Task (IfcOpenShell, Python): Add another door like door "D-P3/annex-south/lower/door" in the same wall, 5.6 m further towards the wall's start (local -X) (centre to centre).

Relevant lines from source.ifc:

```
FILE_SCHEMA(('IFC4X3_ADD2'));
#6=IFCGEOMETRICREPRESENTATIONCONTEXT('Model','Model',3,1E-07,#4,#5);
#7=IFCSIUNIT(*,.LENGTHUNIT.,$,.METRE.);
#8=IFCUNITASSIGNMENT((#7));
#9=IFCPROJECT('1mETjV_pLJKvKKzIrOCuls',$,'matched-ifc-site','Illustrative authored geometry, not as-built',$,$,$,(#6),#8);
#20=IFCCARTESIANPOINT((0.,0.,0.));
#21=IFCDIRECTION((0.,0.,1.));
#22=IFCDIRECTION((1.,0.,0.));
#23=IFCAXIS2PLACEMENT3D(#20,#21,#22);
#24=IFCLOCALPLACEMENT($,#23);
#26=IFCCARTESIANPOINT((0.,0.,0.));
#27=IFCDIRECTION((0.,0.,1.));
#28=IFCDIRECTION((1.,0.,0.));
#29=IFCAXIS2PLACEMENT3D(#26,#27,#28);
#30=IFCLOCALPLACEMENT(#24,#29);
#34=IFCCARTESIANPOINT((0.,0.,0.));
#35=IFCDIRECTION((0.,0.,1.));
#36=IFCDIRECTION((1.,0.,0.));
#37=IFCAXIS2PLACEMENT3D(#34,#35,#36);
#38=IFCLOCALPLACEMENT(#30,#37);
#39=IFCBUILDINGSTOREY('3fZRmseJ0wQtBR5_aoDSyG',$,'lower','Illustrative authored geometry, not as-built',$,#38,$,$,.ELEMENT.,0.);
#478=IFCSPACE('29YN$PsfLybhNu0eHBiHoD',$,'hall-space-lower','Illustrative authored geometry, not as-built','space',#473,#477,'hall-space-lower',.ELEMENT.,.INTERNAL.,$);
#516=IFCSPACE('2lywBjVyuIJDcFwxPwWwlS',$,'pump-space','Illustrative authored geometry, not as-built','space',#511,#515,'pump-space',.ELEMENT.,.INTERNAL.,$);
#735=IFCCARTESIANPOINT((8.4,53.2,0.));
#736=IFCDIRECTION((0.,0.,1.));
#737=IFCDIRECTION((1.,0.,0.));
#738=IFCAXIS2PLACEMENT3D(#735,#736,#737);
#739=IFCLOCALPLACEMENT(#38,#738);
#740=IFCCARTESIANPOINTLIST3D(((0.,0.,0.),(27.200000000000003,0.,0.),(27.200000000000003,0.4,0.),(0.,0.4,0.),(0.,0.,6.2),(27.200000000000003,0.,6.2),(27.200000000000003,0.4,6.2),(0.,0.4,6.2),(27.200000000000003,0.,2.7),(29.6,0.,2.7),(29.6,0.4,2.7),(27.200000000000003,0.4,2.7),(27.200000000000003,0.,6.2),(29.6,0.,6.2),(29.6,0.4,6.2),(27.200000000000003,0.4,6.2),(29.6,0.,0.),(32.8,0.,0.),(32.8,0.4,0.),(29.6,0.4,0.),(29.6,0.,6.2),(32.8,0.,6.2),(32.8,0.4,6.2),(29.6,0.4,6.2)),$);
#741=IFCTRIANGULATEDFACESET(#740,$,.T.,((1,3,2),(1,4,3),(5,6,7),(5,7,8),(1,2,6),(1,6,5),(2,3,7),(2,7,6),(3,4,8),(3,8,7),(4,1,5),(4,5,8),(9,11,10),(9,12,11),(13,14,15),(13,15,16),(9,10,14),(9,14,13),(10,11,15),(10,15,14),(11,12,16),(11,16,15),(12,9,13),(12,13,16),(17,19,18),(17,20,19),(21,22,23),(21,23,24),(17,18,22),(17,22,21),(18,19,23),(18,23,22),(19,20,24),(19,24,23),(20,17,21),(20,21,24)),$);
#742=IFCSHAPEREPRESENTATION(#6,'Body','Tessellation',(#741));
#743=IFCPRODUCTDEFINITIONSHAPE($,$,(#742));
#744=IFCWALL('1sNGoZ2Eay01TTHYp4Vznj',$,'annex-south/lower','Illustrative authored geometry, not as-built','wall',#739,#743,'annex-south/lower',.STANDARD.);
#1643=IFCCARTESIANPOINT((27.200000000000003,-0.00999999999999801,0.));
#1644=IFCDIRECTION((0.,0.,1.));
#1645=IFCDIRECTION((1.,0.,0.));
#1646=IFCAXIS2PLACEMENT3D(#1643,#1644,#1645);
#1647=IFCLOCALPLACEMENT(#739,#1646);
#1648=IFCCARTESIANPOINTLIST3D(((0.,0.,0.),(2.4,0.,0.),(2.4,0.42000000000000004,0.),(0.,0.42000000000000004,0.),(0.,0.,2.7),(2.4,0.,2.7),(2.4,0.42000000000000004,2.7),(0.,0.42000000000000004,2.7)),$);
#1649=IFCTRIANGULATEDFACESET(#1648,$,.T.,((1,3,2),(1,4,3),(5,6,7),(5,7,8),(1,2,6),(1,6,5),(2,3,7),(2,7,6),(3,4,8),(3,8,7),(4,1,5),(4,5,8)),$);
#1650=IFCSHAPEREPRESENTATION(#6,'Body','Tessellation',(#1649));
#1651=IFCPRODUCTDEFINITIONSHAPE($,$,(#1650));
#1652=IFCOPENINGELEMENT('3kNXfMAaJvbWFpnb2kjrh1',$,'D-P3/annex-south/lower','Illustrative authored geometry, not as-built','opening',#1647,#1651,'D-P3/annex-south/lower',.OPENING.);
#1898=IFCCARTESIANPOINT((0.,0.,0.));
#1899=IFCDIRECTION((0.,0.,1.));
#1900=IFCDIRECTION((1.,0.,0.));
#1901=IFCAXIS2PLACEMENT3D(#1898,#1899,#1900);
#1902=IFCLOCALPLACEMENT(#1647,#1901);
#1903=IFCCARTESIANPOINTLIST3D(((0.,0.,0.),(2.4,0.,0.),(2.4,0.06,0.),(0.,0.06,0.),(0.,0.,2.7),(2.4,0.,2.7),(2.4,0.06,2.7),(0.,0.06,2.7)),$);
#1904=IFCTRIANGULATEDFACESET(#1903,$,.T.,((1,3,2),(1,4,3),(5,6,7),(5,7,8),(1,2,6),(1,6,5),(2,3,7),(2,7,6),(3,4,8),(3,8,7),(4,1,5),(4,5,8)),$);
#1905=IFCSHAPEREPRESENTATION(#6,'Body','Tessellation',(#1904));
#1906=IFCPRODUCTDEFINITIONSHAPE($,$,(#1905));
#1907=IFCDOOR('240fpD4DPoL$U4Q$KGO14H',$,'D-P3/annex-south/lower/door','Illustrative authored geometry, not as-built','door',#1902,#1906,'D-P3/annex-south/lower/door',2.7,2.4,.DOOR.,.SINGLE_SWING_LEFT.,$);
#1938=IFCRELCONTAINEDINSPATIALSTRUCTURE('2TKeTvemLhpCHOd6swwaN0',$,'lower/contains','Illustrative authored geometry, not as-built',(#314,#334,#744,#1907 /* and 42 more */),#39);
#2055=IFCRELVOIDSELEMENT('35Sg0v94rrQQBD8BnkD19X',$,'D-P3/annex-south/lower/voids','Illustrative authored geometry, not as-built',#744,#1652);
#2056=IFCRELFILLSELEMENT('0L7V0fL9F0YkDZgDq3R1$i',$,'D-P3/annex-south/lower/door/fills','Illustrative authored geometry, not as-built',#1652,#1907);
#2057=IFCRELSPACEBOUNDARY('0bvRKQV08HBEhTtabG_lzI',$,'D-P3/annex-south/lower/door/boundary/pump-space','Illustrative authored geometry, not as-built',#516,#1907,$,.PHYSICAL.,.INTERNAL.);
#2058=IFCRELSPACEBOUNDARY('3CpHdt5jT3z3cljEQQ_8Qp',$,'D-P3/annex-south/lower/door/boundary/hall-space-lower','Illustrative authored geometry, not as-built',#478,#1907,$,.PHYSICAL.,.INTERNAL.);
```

```python
import ifcopenshell
import ifcopenshell.api.feature
import ifcopenshell.api.geometry
import ifcopenshell.api.root
import ifcopenshell.geom
import ifcopenshell.util.element
import ifcopenshell.util.placement
import ifcopenshell.util.shape

model = ifcopenshell.open("source.ifc")
settings = ifcopenshell.geom.settings()


def volume(element):
    """Net volume in cubic metres, openings subtracted."""
    shape = ifcopenshell.geom.create_shape(settings, element)
    return ifcopenshell.util.shape.get_volume(shape.geometry)


door = model.by_guid("240fpD4DPoL$U4Q$KGO14H")
opening = door.FillsVoids[0].RelatingOpeningElement
wall = opening.VoidsElements[0].RelatingBuildingElement
before = volume(wall)
shift = ifcopenshell.util.placement.get_local_placement(wall.ObjectPlacement)[:3, 0] * -5.6

# copy_class copies the void relationship, type, container and properties, but no geometry.
new_opening = ifcopenshell.api.root.copy_class(model, product=opening)
new_opening.Representation = ifcopenshell.util.element.copy_deep(
    model, opening.Representation, exclude=["IfcGeometricRepresentationContext", "IfcRepresentationMap"]
)
new_opening.Tag = None
new_door = ifcopenshell.api.root.copy_class(model, product=door)
new_door.Representation = ifcopenshell.util.element.copy_deep(
    model, door.Representation, exclude=["IfcGeometricRepresentationContext", "IfcRepresentationMap"]
)
new_door.Tag = None
ifcopenshell.api.feature.add_filling(model, opening=new_opening, element=new_door)

for old, new in ((opening, new_opening), (door, new_door)):
    matrix = ifcopenshell.util.placement.get_local_placement(old.ObjectPlacement)
    matrix[:3, 3] += shift
    ifcopenshell.api.geometry.edit_object_placement(model, product=new, matrix=matrix, is_si=False)

after = volume(wall)

print(f"wall volume {before:.3f} -> {after:.3f} m3")

model.write("source_v2.ifc")
```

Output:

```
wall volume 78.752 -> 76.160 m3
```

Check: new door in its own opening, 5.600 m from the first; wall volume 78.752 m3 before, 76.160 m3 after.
